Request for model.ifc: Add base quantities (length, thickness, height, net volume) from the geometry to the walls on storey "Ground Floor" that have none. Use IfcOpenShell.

First a look at what the model holds.

```python
import ifcopenshell
import ifcopenshell.util.element
import ifcopenshell.util.unit

model = ifcopenshell.open("model.ifc")
print(model.schema)
for unit_type in ("LENGTHUNIT", "AREAUNIT", "VOLUMEUNIT"):
    print(unit_type, ifcopenshell.util.unit.calculate_unit_scale(model, unit_type))
storey = next(s for s in model.by_type("IfcBuildingStorey") if s.Name == "Ground Floor")
walls = [e for e in ifcopenshell.util.element.get_decomposition(storey) if e.is_a("IfcWall")]
for e in sorted(walls, key=lambda e: e.id()):
    print(e.id(), e.is_a(), e.Name, list(ifcopenshell.util.element.get_psets(e, qtos_only=True)), sep=" | ")
```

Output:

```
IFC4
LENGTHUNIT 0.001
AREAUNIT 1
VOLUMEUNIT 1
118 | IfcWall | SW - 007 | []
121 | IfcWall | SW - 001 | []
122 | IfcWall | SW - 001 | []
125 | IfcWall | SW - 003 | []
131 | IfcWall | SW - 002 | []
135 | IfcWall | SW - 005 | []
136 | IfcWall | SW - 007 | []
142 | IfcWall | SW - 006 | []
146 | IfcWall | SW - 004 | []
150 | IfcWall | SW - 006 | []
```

```python
import ifcopenshell
import ifcopenshell.api.pset
import ifcopenshell.geom
import ifcopenshell.util.element
import ifcopenshell.util.shape
import ifcopenshell.util.unit

model = ifcopenshell.open("model.ifc")
unit_scale = ifcopenshell.util.unit.calculate_unit_scale(model)
volume_scale = ifcopenshell.util.unit.calculate_unit_scale(model, "VOLUMEUNIT")
settings = ifcopenshell.geom.settings()

storey = next(s for s in model.by_type("IfcBuildingStorey") if s.Name == "Ground Floor")
walls = [e for e in ifcopenshell.util.element.get_decomposition(storey) if e.is_a("IfcWall")]

for e in sorted(walls, key=lambda e: e.id()):
    if ifcopenshell.util.element.get_psets(e, qtos_only=True, should_inherit=False):
        continue
    # Geometry comes back in metres, in the element's own axes.
    shape = ifcopenshell.geom.create_shape(settings, e)
    values = {
        "Length": ifcopenshell.util.shape.get_x(shape.geometry) / unit_scale,
        "Width": ifcopenshell.util.shape.get_y(shape.geometry) / unit_scale,
        "Height": ifcopenshell.util.shape.get_z(shape.geometry) / unit_scale,
        "NetVolume": ifcopenshell.util.shape.get_volume(shape.geometry) / volume_scale,
    }
    qto = ifcopenshell.api.pset.add_qto(model, product=e, name="Qto_WallBaseQuantities")
    ifcopenshell.api.pset.edit_qto(model, qto=qto, properties=values)
    print(e.id(), {k: round(v, 3) for k, v in values.items()})

model.write("model_v2.ifc")
```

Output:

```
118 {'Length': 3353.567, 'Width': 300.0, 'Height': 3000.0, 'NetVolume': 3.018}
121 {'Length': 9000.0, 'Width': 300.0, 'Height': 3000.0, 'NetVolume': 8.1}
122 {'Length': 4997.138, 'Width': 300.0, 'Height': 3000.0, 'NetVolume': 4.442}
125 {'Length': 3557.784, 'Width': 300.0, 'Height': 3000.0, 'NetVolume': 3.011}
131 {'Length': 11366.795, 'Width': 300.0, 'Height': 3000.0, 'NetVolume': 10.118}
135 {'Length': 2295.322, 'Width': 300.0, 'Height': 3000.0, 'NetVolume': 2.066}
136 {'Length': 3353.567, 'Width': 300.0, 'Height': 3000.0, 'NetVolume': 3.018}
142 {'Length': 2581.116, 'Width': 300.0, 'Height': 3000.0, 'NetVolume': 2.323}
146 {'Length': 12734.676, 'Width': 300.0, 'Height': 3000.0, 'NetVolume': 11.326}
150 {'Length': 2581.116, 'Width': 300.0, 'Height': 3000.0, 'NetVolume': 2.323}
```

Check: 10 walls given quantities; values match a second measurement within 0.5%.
